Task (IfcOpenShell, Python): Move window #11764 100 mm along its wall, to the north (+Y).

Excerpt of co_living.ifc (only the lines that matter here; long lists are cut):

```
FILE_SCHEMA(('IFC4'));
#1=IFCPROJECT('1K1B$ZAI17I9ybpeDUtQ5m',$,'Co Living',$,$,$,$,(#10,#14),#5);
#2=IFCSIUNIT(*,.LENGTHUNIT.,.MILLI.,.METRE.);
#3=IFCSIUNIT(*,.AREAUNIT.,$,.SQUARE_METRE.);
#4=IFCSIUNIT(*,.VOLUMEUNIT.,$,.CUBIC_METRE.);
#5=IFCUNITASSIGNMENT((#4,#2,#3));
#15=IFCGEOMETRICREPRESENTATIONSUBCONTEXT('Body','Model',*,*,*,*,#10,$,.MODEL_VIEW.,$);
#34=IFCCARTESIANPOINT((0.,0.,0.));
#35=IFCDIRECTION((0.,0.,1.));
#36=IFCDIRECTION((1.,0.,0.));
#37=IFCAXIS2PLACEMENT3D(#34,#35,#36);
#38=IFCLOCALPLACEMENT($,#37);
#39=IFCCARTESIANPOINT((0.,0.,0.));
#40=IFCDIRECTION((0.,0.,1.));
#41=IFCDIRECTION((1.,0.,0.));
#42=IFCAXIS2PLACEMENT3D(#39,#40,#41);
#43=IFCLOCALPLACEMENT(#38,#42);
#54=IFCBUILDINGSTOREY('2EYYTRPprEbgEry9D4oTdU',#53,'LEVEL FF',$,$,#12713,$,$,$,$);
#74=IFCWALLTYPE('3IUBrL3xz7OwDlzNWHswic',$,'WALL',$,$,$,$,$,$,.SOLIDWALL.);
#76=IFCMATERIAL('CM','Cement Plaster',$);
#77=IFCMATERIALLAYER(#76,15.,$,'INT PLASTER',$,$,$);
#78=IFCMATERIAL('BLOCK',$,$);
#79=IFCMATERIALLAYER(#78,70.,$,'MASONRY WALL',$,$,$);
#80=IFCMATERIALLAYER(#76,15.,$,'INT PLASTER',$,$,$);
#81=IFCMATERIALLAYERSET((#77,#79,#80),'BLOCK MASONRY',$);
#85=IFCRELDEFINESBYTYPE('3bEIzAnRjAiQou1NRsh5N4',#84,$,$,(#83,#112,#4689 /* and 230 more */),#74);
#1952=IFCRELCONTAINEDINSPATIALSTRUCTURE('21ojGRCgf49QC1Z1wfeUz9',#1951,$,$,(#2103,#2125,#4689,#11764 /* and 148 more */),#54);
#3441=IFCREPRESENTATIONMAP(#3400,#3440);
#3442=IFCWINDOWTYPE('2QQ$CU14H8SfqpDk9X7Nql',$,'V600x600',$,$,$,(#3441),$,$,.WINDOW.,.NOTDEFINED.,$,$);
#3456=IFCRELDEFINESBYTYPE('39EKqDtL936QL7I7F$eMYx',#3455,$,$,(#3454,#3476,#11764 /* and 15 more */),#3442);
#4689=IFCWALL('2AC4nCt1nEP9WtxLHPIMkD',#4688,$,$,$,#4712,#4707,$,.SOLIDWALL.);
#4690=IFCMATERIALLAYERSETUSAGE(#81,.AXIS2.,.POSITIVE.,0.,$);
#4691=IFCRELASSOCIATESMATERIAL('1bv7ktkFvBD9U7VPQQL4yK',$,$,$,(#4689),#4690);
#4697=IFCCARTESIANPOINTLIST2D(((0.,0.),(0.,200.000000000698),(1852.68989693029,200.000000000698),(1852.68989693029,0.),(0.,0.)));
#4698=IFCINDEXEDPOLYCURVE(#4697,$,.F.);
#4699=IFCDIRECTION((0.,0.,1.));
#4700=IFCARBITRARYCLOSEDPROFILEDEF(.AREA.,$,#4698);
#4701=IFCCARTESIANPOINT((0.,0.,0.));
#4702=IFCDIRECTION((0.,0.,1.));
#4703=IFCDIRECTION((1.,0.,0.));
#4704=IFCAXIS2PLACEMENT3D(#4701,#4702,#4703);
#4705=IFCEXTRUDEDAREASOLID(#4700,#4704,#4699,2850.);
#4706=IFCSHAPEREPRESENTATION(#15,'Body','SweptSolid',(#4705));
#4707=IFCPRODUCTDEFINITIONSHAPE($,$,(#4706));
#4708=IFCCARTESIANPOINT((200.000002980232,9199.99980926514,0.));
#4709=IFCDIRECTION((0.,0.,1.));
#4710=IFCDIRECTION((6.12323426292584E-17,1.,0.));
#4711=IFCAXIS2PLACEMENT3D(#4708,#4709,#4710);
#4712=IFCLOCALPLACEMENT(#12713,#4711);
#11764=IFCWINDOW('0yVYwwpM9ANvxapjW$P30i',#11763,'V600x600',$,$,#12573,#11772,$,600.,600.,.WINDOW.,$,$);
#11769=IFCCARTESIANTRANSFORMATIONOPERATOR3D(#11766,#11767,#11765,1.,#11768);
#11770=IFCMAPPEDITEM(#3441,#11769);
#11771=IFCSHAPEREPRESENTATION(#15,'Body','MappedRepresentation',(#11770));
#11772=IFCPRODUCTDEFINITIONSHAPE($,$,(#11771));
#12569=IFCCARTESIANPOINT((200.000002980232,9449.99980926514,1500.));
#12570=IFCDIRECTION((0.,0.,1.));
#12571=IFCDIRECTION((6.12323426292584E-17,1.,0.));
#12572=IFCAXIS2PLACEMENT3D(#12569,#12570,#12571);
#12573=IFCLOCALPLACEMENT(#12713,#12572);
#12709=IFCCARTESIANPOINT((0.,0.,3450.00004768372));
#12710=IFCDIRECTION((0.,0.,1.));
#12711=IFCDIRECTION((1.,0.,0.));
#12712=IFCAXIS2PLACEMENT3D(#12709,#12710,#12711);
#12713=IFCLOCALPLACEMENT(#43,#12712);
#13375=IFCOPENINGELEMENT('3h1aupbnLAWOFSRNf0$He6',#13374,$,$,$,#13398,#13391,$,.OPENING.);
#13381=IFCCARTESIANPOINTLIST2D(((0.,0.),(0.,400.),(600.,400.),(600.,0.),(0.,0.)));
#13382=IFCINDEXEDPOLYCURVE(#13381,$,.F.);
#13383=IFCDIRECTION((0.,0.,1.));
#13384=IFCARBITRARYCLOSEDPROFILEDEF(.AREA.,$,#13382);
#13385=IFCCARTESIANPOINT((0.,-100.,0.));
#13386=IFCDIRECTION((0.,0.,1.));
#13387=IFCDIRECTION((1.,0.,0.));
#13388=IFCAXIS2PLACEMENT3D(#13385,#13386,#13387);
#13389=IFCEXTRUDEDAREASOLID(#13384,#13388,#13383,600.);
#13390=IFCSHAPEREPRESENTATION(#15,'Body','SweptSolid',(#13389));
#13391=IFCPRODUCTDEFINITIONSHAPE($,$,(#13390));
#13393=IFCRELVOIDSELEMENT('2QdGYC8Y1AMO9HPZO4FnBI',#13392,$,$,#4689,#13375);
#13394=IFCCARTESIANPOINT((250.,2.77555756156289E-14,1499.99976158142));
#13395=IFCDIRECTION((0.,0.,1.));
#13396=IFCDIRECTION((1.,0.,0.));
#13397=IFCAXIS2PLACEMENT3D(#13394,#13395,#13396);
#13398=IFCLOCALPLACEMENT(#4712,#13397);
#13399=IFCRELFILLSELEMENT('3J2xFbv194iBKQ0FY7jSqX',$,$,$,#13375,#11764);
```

```python
import ifcopenshell
import ifcopenshell.api.geometry
import ifcopenshell.util.placement

model = ifcopenshell.open("co_living.ifc")

window = model.by_guid("0yVYwwpM9ANvxapjW$P30i")
opening = window.FillsVoids[0].RelatingOpeningElement
wall = opening.VoidsElements[0].RelatingBuildingElement

wall_matrix = ifcopenshell.util.placement.get_local_placement(wall.ObjectPlacement)
shift = wall_matrix[:3, 0] * 100.0
before = ifcopenshell.util.placement.get_local_placement(window.ObjectPlacement)[:3, 3].copy()

# The window is not placed relative to its opening, so move both.
for product in (opening, window):
    matrix = ifcopenshell.util.placement.get_local_placement(product.ObjectPlacement)
    matrix[:3, 3] += shift
    ifcopenshell.api.geometry.edit_object_placement(model, product=product, matrix=matrix, is_si=False)

after = ifcopenshell.util.placement.get_local_placement(window.ObjectPlacement)[:3, 3]
print("window moved by", (after - before).round(3) + 0.0)

model.write("co_living_updated.ifc")
```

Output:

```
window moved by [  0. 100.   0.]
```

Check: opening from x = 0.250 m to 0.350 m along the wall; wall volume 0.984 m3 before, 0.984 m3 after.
